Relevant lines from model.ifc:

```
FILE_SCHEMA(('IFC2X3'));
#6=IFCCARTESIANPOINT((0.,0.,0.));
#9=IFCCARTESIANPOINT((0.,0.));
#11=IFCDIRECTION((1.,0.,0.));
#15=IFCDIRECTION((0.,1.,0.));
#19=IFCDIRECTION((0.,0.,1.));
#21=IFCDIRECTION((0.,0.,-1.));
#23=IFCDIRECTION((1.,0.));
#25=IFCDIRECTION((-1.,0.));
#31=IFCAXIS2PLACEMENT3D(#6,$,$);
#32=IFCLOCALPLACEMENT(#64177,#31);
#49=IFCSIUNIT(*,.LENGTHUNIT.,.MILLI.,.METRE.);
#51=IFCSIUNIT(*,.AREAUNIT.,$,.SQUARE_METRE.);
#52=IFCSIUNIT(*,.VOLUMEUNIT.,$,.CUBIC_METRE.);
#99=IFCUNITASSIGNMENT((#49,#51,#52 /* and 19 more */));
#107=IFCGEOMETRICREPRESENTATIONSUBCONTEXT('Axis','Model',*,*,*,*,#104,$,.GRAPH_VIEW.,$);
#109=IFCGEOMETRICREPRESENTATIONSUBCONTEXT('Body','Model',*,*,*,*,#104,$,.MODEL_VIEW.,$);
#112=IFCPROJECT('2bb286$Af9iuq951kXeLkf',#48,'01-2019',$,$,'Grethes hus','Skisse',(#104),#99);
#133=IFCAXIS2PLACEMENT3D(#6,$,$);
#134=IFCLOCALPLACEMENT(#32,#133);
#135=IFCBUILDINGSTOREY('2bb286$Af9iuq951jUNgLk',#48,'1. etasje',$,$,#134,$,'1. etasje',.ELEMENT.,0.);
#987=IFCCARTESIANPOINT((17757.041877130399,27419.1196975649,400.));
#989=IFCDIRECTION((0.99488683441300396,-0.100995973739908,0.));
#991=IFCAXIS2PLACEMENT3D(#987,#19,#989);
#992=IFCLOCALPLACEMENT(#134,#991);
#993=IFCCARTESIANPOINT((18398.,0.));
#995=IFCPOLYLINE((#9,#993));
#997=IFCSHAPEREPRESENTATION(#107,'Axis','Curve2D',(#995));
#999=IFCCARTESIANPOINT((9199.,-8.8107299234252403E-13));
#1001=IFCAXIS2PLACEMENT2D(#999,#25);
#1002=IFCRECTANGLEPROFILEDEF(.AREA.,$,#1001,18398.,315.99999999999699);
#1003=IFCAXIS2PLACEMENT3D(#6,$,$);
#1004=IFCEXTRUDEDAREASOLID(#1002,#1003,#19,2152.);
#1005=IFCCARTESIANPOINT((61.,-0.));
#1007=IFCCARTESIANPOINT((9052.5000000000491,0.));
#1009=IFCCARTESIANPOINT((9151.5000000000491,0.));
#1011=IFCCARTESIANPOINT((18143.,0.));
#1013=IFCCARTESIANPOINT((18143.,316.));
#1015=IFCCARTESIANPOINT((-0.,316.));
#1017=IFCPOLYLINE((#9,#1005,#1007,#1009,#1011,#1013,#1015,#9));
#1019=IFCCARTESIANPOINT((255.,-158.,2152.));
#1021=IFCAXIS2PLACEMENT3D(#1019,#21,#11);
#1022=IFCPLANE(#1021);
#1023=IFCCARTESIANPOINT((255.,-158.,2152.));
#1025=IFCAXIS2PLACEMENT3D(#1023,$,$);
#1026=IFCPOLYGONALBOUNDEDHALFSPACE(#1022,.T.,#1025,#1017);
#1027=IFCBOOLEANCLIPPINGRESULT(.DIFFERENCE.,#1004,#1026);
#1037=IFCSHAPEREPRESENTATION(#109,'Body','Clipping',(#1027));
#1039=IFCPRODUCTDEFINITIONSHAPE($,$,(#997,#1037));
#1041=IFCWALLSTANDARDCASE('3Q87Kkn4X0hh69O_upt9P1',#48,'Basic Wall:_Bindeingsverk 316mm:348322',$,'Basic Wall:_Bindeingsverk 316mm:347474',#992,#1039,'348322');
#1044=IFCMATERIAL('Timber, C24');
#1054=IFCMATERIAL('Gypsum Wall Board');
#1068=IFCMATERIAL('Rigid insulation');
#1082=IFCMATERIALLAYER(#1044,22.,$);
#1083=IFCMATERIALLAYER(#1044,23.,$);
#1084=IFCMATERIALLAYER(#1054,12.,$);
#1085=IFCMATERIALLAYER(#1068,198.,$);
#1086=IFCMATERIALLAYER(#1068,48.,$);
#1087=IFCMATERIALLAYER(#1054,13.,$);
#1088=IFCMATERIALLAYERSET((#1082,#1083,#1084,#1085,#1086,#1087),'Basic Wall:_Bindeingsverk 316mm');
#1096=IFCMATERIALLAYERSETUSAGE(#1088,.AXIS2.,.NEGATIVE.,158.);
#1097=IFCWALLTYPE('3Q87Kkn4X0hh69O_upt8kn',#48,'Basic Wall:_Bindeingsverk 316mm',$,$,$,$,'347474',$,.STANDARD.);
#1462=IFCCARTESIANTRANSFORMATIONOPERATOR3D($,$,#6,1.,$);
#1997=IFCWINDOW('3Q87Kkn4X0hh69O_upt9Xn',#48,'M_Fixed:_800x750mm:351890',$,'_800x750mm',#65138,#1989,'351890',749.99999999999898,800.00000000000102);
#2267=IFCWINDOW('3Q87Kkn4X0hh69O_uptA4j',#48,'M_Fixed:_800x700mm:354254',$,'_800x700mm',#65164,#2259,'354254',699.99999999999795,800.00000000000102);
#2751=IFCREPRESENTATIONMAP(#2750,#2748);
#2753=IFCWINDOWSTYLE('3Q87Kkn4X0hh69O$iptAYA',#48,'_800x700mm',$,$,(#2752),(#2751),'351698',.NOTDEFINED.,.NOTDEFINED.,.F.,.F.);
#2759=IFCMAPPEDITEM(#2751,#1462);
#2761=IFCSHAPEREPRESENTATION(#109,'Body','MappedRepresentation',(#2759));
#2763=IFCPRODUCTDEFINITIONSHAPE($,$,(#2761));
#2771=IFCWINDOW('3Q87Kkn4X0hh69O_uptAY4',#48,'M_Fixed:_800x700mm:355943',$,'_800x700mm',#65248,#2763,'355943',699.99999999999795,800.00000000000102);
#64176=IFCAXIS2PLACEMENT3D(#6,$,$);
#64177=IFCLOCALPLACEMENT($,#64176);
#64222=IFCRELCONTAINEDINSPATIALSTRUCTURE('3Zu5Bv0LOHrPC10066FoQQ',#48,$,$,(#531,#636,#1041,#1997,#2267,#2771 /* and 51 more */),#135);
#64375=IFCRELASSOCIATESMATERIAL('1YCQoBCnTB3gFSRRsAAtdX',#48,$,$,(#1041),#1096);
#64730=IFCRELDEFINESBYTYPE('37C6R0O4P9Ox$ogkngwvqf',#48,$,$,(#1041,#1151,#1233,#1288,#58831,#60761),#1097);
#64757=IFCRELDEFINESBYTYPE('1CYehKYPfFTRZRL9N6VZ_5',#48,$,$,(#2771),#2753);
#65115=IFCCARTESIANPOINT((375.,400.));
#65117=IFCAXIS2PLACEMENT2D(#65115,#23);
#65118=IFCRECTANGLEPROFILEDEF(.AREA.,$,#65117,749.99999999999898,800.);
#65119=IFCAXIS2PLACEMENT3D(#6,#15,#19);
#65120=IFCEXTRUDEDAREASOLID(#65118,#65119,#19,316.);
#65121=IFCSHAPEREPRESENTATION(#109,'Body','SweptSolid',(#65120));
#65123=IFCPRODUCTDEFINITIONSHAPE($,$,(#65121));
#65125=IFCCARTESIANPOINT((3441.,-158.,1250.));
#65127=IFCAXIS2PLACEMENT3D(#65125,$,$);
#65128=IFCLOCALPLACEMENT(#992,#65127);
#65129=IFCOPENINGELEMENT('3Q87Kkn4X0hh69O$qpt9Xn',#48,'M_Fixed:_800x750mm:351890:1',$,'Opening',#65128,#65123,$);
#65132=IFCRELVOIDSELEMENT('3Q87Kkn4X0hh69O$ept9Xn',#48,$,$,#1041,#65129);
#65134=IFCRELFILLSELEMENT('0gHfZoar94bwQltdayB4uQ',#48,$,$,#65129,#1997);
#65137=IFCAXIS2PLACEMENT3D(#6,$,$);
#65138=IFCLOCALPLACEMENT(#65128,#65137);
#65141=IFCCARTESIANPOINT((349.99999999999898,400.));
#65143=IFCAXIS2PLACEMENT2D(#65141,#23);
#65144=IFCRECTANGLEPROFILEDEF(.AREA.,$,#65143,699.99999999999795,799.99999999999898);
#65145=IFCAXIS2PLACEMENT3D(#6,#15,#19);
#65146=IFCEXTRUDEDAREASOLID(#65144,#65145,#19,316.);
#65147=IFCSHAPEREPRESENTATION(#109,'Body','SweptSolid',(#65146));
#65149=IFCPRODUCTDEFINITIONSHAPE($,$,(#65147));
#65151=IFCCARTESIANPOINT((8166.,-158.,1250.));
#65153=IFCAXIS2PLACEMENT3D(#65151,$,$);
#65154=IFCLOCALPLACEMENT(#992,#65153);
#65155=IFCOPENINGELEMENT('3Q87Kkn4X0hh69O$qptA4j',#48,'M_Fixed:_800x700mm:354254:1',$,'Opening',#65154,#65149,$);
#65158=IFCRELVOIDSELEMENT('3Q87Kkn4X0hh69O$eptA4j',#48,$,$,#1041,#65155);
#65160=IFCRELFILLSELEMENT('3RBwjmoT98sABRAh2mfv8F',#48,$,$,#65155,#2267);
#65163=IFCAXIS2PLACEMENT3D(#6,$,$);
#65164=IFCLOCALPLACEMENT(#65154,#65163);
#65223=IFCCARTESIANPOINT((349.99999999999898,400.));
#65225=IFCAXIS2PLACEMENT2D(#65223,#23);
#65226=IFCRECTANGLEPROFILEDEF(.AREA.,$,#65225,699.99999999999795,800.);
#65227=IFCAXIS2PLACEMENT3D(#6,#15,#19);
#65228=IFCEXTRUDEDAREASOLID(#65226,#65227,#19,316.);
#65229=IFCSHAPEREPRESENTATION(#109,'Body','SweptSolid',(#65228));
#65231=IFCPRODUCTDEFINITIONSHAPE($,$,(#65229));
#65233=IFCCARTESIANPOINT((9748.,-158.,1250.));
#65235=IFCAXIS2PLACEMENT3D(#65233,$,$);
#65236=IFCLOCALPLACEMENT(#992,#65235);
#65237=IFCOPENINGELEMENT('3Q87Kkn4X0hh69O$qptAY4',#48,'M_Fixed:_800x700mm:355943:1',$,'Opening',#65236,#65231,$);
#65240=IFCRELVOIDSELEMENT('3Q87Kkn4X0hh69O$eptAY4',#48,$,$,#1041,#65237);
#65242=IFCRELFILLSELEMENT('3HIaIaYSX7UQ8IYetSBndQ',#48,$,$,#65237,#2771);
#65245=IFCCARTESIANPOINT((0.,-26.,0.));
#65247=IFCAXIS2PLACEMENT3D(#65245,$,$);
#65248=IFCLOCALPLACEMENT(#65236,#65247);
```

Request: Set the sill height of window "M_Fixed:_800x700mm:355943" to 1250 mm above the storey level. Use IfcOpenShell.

```python
import numpy as np
import ifcopenshell
import ifcopenshell.api.geometry
import ifcopenshell.geom
import ifcopenshell.util.element
import ifcopenshell.util.placement
import ifcopenshell.util.shape
import ifcopenshell.util.unit

model = ifcopenshell.open("model.ifc")
unit_scale = ifcopenshell.util.unit.calculate_unit_scale(model)

window = model.by_guid("3Q87Kkn4X0hh69O_uptAY4")
opening = window.FillsVoids[0].RelatingOpeningElement
storey = ifcopenshell.util.element.get_container(window, ifc_class="IfcBuildingStorey")
level = ifcopenshell.util.placement.get_local_placement(storey.ObjectPlacement)[2, 3]

# The opening's origin need not be at the sill, so measure its lowest point.
shape = ifcopenshell.geom.create_shape(ifcopenshell.geom.settings(), opening)
bottom = ifcopenshell.util.shape.get_shape_bottom_elevation(shape, shape.geometry) / unit_scale
dz = level + 1.25 / unit_scale - bottom

shift = np.array([0.0, 0.0, dz])
# The window is placed relative to its opening, so it follows when the opening moves.
matrix = ifcopenshell.util.placement.get_local_placement(opening.ObjectPlacement)
matrix[:3, 3] += shift
ifcopenshell.api.geometry.edit_object_placement(
    model, product=opening, matrix=matrix, is_si=False, should_transform_children=True
)

print(f"moved by {dz * unit_scale:+.3f} m")

model.write("model_edited.ifc")
```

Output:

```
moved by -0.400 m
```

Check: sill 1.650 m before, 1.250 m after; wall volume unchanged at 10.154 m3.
